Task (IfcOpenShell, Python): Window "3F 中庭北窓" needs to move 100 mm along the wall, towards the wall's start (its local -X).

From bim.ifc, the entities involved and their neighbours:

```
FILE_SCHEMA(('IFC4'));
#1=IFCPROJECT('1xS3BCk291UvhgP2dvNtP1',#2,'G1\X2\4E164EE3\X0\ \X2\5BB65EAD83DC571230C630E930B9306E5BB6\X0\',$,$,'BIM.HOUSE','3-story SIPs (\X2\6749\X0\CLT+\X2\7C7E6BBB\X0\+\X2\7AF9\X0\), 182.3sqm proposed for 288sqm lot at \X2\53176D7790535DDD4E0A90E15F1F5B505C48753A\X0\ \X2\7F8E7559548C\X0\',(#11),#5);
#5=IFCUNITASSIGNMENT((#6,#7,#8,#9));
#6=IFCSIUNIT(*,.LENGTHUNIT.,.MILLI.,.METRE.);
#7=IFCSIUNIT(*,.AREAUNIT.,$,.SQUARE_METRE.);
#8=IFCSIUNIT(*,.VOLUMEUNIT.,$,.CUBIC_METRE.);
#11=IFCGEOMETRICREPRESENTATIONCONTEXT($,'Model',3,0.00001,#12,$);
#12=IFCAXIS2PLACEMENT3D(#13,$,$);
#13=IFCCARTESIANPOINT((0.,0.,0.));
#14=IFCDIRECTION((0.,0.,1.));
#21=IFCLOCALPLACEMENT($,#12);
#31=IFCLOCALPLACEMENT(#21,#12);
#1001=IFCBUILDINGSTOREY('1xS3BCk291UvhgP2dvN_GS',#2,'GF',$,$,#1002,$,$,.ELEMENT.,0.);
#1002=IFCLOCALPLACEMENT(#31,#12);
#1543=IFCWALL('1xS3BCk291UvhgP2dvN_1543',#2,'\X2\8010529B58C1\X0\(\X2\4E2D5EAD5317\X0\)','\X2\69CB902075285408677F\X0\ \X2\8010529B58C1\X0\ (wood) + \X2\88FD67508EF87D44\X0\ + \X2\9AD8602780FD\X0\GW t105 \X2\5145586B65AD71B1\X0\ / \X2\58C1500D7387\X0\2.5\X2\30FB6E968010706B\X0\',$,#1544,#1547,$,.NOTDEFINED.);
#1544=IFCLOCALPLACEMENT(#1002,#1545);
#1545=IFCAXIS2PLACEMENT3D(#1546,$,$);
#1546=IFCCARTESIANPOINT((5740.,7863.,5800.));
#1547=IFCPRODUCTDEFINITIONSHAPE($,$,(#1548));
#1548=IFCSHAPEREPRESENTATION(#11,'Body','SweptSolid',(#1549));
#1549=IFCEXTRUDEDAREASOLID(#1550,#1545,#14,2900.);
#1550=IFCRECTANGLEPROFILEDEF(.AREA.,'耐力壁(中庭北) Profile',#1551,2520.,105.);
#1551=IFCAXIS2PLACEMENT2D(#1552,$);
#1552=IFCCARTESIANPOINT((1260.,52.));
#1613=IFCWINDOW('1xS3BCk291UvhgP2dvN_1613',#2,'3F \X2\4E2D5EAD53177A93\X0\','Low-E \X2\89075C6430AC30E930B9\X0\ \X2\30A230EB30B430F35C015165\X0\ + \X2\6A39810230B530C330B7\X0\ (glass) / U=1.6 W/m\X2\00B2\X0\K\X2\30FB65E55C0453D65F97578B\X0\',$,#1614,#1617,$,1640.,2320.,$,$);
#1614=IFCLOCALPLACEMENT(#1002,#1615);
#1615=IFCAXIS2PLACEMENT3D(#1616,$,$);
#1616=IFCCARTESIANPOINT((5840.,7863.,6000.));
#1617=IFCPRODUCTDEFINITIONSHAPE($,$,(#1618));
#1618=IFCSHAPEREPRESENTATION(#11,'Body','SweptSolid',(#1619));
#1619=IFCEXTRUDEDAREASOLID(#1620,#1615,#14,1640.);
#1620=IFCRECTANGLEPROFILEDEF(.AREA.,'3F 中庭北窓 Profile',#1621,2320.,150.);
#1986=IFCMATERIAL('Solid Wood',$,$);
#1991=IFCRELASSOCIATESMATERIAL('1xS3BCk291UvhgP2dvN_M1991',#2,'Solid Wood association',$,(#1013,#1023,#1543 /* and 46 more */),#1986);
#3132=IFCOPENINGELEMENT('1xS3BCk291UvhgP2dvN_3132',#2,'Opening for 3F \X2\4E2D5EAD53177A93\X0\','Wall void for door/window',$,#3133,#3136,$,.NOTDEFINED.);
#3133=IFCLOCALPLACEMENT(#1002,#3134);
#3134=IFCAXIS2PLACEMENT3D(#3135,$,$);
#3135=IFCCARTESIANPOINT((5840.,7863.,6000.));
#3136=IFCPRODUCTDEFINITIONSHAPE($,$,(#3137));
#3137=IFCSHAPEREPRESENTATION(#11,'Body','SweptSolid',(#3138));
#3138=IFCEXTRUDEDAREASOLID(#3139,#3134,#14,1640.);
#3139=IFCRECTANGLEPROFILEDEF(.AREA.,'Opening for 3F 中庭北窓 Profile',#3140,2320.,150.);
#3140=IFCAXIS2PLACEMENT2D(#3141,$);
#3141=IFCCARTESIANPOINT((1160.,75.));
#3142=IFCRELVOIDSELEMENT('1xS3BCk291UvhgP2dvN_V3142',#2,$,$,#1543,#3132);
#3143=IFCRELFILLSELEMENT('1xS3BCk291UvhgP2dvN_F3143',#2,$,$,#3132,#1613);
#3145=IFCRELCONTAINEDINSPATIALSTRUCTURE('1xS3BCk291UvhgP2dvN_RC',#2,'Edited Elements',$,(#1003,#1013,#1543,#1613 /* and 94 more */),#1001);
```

```python
import ifcopenshell
import ifcopenshell.api.geometry
import ifcopenshell.util.placement

model = ifcopenshell.open("bim.ifc")

window = model.by_guid("1xS3BCk291UvhgP2dvN_1613")
opening = window.FillsVoids[0].RelatingOpeningElement
wall = opening.VoidsElements[0].RelatingBuildingElement

wall_matrix = ifcopenshell.util.placement.get_local_placement(wall.ObjectPlacement)
shift = wall_matrix[:3, 0] * -100.0
before = ifcopenshell.util.placement.get_local_placement(window.ObjectPlacement)[:3, 3].copy()

# The window is not placed relative to its opening, so move both.
for product in (opening, window):
    matrix = ifcopenshell.util.placement.get_local_placement(product.ObjectPlacement)
    matrix[:3, 3] += shift
    ifcopenshell.api.geometry.edit_object_placement(model, product=product, matrix=matrix, is_si=False)

after = ifcopenshell.util.placement.get_local_placement(window.ObjectPlacement)[:3, 3]
print("window moved by", (after - before).round(3) + 0.0)

model.write("bim_rev.ifc")
```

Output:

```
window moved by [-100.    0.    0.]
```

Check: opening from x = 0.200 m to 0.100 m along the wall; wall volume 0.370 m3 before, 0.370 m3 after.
